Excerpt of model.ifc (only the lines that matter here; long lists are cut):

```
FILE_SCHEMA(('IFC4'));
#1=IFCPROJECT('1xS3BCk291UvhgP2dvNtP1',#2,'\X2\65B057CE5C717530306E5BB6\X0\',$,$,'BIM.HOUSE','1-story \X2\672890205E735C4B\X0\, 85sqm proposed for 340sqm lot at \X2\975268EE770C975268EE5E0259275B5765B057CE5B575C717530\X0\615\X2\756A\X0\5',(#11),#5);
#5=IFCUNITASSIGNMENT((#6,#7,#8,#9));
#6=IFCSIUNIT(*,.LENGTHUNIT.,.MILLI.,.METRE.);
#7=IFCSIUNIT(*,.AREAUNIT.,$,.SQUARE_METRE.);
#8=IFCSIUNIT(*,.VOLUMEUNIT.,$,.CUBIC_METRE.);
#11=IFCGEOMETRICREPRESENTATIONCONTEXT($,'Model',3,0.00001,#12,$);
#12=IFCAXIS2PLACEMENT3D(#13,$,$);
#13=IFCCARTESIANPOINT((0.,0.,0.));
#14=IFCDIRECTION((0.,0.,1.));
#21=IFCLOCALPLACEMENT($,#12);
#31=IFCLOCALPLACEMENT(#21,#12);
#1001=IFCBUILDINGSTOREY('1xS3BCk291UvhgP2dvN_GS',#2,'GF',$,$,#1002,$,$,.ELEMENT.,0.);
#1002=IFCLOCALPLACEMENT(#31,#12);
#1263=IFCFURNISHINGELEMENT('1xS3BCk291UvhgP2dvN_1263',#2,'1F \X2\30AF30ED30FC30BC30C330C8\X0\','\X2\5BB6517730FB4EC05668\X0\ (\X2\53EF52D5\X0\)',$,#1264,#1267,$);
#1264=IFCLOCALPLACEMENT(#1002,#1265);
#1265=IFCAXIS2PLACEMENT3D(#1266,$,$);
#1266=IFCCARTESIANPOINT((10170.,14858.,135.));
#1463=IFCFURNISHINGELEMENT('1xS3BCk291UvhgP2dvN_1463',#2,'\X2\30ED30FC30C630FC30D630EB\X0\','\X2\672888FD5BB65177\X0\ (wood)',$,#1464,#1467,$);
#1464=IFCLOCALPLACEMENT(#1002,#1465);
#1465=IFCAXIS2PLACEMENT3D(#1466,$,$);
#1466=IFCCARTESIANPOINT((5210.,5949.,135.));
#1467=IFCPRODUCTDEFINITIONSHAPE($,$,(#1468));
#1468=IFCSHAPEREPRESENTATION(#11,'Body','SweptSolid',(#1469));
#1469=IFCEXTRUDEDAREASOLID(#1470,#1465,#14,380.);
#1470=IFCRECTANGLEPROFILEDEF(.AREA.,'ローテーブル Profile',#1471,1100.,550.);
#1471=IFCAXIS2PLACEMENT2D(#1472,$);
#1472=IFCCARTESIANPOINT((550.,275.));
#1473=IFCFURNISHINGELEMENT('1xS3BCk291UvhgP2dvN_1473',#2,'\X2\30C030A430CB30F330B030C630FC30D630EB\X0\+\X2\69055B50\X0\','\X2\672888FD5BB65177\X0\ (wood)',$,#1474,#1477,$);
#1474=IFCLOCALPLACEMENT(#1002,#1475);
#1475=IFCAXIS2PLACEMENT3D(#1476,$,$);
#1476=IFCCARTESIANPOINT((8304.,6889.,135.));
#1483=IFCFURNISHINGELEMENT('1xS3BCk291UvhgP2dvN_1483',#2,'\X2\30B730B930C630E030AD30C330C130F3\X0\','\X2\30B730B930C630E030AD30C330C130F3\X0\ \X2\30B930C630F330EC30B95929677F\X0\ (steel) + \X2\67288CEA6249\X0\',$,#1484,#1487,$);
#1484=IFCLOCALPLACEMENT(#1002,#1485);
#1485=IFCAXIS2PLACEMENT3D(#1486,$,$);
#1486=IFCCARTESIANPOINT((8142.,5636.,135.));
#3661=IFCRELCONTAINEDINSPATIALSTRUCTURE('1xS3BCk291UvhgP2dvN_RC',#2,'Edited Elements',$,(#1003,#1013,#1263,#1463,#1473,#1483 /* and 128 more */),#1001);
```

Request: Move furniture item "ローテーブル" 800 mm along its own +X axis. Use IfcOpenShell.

```python
import ifcopenshell
import ifcopenshell.api.geometry
import ifcopenshell.util.placement

model = ifcopenshell.open("model.ifc")

item = model.by_guid("1xS3BCk291UvhgP2dvN_1463")
matrix = ifcopenshell.util.placement.get_local_placement(item.ObjectPlacement)
matrix[:3, 3] += matrix[:3, 0] * 800.0
ifcopenshell.api.geometry.edit_object_placement(model, product=item, matrix=matrix, is_si=False)

print(ifcopenshell.util.placement.get_local_placement(item.ObjectPlacement).round(3) + 0.0)

model.write("model_edited.ifc")
```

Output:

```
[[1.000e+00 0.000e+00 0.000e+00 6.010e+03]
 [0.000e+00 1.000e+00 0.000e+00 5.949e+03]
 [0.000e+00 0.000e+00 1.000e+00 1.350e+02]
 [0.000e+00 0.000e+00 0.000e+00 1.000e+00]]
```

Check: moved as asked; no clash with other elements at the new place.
